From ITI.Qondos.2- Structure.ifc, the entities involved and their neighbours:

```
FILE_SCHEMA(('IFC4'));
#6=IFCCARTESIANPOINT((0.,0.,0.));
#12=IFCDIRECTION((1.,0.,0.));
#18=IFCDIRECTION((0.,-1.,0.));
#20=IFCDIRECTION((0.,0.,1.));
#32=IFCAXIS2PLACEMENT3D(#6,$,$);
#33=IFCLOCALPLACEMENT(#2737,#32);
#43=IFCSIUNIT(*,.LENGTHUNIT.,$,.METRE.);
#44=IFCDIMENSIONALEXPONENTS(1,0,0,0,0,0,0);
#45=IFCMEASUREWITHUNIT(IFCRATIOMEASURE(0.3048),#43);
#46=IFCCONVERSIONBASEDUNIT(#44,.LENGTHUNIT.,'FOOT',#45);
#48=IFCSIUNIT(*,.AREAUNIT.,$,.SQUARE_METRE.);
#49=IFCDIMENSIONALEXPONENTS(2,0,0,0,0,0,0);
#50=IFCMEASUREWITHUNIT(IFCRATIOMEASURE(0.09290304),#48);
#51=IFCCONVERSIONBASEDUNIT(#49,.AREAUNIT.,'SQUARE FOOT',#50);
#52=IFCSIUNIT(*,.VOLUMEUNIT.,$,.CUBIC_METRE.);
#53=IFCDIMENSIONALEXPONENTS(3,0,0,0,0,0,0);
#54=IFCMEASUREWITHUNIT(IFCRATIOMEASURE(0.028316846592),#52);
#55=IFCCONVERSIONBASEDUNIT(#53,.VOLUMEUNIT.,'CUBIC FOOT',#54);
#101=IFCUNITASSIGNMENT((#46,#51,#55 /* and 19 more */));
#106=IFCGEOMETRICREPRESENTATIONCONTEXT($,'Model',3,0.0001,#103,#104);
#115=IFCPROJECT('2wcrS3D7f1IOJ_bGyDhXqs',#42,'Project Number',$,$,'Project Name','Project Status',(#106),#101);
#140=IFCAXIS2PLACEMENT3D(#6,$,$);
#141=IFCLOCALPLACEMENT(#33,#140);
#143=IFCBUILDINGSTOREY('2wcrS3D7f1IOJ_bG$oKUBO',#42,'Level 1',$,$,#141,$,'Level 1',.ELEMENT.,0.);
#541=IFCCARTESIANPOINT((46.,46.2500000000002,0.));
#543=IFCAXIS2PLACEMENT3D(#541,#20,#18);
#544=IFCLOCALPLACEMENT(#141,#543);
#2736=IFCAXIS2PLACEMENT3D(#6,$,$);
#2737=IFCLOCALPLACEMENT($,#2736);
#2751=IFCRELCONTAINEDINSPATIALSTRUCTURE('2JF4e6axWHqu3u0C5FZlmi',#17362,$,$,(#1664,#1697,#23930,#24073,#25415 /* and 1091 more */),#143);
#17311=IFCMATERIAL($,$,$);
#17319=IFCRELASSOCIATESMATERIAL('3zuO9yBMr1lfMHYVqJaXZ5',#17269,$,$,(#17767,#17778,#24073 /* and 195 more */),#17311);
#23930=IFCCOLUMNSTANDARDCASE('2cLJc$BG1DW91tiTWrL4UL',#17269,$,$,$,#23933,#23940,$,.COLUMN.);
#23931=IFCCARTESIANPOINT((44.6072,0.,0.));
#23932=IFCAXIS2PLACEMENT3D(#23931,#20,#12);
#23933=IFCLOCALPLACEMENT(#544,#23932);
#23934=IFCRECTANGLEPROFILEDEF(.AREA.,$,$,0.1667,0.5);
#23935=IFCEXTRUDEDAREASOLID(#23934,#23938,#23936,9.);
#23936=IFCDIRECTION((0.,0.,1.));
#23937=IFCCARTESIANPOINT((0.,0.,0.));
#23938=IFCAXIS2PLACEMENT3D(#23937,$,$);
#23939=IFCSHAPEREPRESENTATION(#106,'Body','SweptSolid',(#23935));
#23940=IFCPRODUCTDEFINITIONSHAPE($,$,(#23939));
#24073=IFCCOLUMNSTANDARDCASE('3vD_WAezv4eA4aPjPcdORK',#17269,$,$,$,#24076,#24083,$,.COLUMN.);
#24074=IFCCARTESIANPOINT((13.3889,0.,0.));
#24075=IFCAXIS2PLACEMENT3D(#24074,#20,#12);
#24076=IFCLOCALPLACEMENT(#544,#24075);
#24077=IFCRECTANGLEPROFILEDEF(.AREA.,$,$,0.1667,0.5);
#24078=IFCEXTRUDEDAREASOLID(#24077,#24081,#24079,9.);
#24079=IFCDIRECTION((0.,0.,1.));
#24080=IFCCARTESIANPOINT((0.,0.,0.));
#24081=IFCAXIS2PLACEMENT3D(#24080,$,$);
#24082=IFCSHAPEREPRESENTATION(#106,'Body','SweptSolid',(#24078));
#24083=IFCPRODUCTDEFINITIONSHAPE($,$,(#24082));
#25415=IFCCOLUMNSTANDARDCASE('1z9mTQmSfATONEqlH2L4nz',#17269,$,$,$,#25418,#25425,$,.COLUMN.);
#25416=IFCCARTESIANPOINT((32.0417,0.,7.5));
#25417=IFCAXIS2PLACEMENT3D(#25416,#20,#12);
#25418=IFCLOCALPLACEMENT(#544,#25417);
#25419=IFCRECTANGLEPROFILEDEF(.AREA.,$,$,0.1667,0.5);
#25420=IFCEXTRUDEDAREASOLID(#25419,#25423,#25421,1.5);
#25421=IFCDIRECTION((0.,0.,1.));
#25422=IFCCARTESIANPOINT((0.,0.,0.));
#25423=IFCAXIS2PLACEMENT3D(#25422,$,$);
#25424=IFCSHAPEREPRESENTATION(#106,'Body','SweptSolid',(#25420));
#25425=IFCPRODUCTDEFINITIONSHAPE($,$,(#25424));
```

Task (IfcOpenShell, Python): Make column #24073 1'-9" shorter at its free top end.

```python
import ifcopenshell
import ifcopenshell.util.unit

model = ifcopenshell.open("ITI.Qondos.2- Structure.ifc")
unit_scale = ifcopenshell.util.unit.calculate_unit_scale(model)

member = model.by_guid("3vD_WAezv4eA4aPjPcdORK")
change = -21 * 0.0254 / unit_scale

# The extrusion runs towards the end named, so only its depth changes.
body = next(r for r in member.Representation.Representations if r.RepresentationIdentifier == "Body")
solid = body.Items[0]
old_length = solid.Depth
solid.Depth += change

print(f"length {old_length:g} -> {solid.Depth:g}")

model.write("ITI.Qondos.2- Structure_v2.ifc")
```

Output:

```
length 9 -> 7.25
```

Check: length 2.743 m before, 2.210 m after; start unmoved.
